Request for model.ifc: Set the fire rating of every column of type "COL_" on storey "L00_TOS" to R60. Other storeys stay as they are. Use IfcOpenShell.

First a look at what the model holds.

```python
import ifcopenshell
import ifcopenshell.util.element

model = ifcopenshell.open("model.ifc")
print(model.schema)
storey = next(s for s in model.by_type("IfcBuildingStorey") if s.Name == "L00_TOS")
columns = [e for e in ifcopenshell.util.element.get_decomposition(storey) if e.is_a("IfcColumn")]
seen = {}
for e in columns:
    element_type = ifcopenshell.util.element.get_type(e)
    key = (element_type.Name if element_type != e and element_type else None, ifcopenshell.util.element.get_pset(e, "Pset_ColumnCommon", "FireRating"))
    seen[key] = seen.get(key, 0) + 1
for (name, value), count in sorted(seen.items(), key=str):
    print(count, "x", name, "|", value)
```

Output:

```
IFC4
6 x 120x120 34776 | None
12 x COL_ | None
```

```python
import ifcopenshell
import ifcopenshell.api.pset
import ifcopenshell.util.element

model = ifcopenshell.open("model.ifc")

storey = next(s for s in model.by_type("IfcBuildingStorey") if s.Name == "L00_TOS")
columns = [e for e in ifcopenshell.util.element.get_decomposition(storey) if e.is_a("IfcColumn")]

count = 0
for e in columns:
    element_type = ifcopenshell.util.element.get_type(e)
    if element_type in (None, e) or element_type.Name != "COL_":
        continue
    # add_pset returns the element's existing set when there is one.
    pset = ifcopenshell.api.pset.add_pset(model, product=e, name="Pset_ColumnCommon")
    ifcopenshell.api.pset.edit_pset(model, pset=pset, properties={"FireRating": "R60"})
    count += 1

print(count, "columns updated")

model.write("model-out.ifc")
```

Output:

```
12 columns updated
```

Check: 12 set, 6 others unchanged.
